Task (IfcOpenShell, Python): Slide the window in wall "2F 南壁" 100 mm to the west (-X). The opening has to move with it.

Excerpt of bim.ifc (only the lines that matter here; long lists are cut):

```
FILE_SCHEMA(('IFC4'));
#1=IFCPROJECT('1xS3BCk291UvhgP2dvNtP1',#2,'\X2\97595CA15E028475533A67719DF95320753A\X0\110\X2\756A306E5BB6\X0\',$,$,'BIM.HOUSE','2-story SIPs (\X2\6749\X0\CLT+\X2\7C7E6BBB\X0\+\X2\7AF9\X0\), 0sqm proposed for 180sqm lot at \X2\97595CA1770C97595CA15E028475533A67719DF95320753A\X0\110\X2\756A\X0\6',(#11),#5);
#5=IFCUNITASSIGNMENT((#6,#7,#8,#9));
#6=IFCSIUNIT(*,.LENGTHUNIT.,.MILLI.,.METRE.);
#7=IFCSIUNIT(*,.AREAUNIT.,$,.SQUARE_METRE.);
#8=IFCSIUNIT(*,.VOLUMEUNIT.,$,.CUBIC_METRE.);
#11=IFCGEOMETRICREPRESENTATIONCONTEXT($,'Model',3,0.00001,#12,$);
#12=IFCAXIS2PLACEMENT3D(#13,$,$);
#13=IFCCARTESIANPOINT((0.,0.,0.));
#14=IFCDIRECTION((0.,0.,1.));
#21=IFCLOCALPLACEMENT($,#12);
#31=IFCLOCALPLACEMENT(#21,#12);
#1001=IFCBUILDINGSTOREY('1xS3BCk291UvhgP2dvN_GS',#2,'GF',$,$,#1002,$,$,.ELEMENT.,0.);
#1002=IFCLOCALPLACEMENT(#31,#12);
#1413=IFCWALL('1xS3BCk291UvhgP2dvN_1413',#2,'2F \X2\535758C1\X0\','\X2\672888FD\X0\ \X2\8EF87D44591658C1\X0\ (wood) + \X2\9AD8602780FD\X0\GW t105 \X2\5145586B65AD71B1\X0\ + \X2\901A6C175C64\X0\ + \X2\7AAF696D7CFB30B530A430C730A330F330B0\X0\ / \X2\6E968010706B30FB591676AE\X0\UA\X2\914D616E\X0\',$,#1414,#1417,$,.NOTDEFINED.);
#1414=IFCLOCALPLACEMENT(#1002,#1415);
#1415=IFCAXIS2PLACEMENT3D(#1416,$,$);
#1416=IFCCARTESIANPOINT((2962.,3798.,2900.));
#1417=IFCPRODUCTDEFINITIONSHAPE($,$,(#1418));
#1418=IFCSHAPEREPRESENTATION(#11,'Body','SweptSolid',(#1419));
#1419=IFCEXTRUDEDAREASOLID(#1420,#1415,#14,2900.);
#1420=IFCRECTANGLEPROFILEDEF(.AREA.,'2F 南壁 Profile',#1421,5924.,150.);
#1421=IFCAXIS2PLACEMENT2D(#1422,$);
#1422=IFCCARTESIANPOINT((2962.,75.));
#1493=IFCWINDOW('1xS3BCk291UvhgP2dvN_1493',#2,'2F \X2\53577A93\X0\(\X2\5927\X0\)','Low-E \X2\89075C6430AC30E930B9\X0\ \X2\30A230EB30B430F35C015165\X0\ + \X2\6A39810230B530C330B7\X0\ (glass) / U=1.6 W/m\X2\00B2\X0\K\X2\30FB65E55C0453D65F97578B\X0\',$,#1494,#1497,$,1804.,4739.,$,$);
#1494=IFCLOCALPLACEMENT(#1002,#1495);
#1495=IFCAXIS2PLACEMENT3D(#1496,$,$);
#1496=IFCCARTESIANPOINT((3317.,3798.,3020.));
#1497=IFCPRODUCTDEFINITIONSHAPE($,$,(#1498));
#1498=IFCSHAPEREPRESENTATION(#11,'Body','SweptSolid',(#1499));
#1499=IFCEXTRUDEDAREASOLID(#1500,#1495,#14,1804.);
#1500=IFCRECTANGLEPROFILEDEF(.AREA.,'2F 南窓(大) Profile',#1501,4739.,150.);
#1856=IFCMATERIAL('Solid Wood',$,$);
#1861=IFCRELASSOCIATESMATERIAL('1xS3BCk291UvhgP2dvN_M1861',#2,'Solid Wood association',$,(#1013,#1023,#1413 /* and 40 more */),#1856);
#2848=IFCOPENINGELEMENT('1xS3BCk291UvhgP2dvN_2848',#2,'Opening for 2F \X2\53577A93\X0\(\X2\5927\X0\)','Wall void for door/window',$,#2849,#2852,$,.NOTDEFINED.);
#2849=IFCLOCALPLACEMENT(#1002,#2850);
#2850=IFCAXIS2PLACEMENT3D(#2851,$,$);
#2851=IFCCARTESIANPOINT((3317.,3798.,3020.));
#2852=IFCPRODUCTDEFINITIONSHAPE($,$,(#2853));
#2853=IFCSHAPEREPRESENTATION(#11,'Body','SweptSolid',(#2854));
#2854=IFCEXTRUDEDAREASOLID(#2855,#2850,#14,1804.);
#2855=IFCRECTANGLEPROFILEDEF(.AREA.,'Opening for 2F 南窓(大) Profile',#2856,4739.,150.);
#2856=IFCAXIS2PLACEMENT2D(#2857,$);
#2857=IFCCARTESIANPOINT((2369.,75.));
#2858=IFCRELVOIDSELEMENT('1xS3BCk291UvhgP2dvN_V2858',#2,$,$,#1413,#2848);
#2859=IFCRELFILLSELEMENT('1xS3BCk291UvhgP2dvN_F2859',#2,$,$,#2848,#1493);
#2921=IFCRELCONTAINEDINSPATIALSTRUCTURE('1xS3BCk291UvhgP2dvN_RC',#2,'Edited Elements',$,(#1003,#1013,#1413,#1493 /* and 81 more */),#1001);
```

```python
import ifcopenshell
import ifcopenshell.api.geometry
import ifcopenshell.util.placement

model = ifcopenshell.open("bim.ifc")

window = model.by_guid("1xS3BCk291UvhgP2dvN_1493")
opening = window.FillsVoids[0].RelatingOpeningElement
wall = opening.VoidsElements[0].RelatingBuildingElement

wall_matrix = ifcopenshell.util.placement.get_local_placement(wall.ObjectPlacement)
shift = wall_matrix[:3, 0] * -100.0
before = ifcopenshell.util.placement.get_local_placement(window.ObjectPlacement)[:3, 3].copy()

# The window is not placed relative to its opening, so move both.
for product in (opening, window):
    matrix = ifcopenshell.util.placement.get_local_placement(product.ObjectPlacement)
    matrix[:3, 3] += shift
    ifcopenshell.api.geometry.edit_object_placement(model, product=product, matrix=matrix, is_si=False)

after = ifcopenshell.util.placement.get_local_placement(window.ObjectPlacement)[:3, 3]
print("window moved by", (after - before).round(3) + 0.0)

model.write("bim_edited.ifc")
```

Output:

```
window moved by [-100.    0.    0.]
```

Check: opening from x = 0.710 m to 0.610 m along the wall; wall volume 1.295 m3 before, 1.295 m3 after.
